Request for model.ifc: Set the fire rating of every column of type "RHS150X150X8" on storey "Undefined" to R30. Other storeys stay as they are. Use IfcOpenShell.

First a look at what the model holds.

```python
import ifcopenshell
import ifcopenshell.util.element

model = ifcopenshell.open("model.ifc")
print(model.schema)
storey = next(s for s in model.by_type("IfcBuildingStorey") if s.Name == "Undefined")
columns = [e for e in ifcopenshell.util.element.get_decomposition(storey) if e.is_a("IfcColumn")]
seen = {}
for e in columns:
    element_type = ifcopenshell.util.element.get_type(e)
    key = (element_type.Name if element_type != e and element_type else None, ifcopenshell.util.element.get_pset(e, "Pset_ColumnCommon", "FireRating"))
    seen[key] = seen.get(key, 0) + 1
for (name, value), count in sorted(seen.items(), key=str):
    print(count, "x", name, "|", value)
```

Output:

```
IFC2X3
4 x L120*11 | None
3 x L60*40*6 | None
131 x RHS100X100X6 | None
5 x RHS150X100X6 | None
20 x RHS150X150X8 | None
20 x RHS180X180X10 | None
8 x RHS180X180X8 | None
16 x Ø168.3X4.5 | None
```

```python
import ifcopenshell
import ifcopenshell.api.pset
import ifcopenshell.util.element

model = ifcopenshell.open("model.ifc")

storey = next(s for s in model.by_type("IfcBuildingStorey") if s.Name == "Undefined")
columns = [e for e in ifcopenshell.util.element.get_decomposition(storey) if e.is_a("IfcColumn")]

count = 0
for e in columns:
    element_type = ifcopenshell.util.element.get_type(e)
    if element_type in (None, e) or element_type.Name != "RHS150X150X8":
        continue
    found = ifcopenshell.util.element.get_pset(e, "Pset_ColumnCommon", should_inherit=False)
    if found:
        pset = model.by_id(found["id"])
        if len(ifcopenshell.util.element.get_elements_by_pset(pset)) > 1:
            pset = ifcopenshell.api.pset.unshare_pset(model, products=[e], pset=pset)[0]
    else:
        pset = ifcopenshell.api.pset.add_pset(model, product=e, name="Pset_ColumnCommon")
    ifcopenshell.api.pset.edit_pset(model, pset=pset, properties={"FireRating": "R30"})
    count += 1

print(count, "columns updated")

model.write("model_rev.ifc")
```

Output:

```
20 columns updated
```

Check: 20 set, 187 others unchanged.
